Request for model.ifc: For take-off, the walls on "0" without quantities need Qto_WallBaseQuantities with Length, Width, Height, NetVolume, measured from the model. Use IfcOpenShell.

First a look at what the model holds.

```python
import ifcopenshell
import ifcopenshell.util.element
import ifcopenshell.util.unit

model = ifcopenshell.open("model.ifc")
print(model.schema)
for unit_type in ("LENGTHUNIT", "AREAUNIT", "VOLUMEUNIT"):
    print(unit_type, ifcopenshell.util.unit.calculate_unit_scale(model, unit_type))
storey = next(s for s in model.by_type("IfcBuildingStorey") if s.Name == "0")
walls = [e for e in ifcopenshell.util.element.get_decomposition(storey) if e.is_a("IfcWall")]
for e in sorted(walls, key=lambda e: e.id()):
    print(e.id(), e.is_a(), e.Name, list(ifcopenshell.util.element.get_psets(e, qtos_only=True)), sep=" | ")
```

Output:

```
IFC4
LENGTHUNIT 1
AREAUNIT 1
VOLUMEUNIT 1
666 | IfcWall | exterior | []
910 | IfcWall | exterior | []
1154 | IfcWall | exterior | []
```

```python
import ifcopenshell
import ifcopenshell.api.pset
import ifcopenshell.geom
import ifcopenshell.util.element
import ifcopenshell.util.shape
import ifcopenshell.util.unit

model = ifcopenshell.open("model.ifc")
unit_scale = ifcopenshell.util.unit.calculate_unit_scale(model)
volume_scale = ifcopenshell.util.unit.calculate_unit_scale(model, "VOLUMEUNIT")
settings = ifcopenshell.geom.settings()

storey = next(s for s in model.by_type("IfcBuildingStorey") if s.Name == "0")
walls = [e for e in ifcopenshell.util.element.get_decomposition(storey) if e.is_a("IfcWall")]

for e in sorted(walls, key=lambda e: e.id()):
    if ifcopenshell.util.element.get_psets(e, qtos_only=True, should_inherit=False):
        continue
    # Geometry comes back in metres, in the element's own axes.
    shape = ifcopenshell.geom.create_shape(settings, e)
    values = {
        "Length": ifcopenshell.util.shape.get_x(shape.geometry) / unit_scale,
        "Width": ifcopenshell.util.shape.get_y(shape.geometry) / unit_scale,
        "Height": ifcopenshell.util.shape.get_z(shape.geometry) / unit_scale,
        "NetVolume": ifcopenshell.util.shape.get_volume(shape.geometry) / volume_scale,
    }
    qto = ifcopenshell.api.pset.add_qto(model, product=e, name="Qto_WallBaseQuantities")
    ifcopenshell.api.pset.edit_qto(model, qto=qto, properties=values)
    print(e.id(), {k: round(v, 3) for k, v in values.items()})

model.write("model_updated.ifc")
```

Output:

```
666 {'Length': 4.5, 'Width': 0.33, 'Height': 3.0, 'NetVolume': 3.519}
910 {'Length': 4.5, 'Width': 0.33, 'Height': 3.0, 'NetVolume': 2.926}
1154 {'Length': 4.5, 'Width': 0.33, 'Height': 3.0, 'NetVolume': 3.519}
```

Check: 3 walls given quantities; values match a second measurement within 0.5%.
